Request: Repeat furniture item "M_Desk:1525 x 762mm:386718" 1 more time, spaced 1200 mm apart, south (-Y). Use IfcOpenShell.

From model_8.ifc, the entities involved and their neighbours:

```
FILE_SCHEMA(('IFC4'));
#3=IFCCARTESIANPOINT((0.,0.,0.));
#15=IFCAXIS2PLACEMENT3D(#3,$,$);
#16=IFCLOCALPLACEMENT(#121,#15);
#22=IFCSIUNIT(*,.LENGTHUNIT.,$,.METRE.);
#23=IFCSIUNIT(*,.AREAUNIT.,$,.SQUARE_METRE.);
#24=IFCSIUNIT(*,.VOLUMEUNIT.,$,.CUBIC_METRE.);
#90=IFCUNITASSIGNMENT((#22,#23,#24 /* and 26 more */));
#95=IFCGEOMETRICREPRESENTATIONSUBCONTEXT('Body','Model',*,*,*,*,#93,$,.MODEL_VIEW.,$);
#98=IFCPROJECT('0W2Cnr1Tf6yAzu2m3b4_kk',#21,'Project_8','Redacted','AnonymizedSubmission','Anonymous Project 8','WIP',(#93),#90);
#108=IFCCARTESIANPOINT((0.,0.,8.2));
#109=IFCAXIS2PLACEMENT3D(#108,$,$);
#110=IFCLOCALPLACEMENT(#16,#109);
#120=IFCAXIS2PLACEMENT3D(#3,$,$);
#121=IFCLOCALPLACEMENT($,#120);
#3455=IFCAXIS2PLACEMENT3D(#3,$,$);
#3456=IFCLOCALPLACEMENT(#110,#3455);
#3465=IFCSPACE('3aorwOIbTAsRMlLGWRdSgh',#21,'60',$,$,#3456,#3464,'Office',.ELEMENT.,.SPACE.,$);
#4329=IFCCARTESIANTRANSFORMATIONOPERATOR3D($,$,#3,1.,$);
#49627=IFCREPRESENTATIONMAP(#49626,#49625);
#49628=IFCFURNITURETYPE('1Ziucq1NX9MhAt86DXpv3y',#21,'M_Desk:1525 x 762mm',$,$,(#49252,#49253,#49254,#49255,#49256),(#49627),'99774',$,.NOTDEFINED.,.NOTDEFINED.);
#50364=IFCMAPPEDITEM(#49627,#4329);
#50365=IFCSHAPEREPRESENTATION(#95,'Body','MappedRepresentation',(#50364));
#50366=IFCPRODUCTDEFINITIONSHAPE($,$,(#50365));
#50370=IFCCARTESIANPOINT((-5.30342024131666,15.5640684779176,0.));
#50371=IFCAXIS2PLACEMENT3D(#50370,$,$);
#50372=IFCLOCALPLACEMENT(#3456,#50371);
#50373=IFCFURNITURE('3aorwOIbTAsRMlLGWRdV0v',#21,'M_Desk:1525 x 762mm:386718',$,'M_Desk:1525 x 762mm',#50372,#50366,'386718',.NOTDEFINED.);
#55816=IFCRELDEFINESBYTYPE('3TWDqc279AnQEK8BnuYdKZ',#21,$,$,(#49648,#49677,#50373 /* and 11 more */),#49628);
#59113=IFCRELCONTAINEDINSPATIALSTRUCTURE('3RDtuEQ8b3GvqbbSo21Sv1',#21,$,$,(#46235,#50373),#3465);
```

```python
import numpy as np
import ifcopenshell
import ifcopenshell.api.geometry
import ifcopenshell.api.root
import ifcopenshell.util.element
import ifcopenshell.util.placement
import ifcopenshell.util.unit

model = ifcopenshell.open("model_8.ifc")
unit_scale = ifcopenshell.util.unit.calculate_unit_scale(model)


def reuse_history(source, copy):
    """copy_class also copies each property set's owner history, people and application; keep the originals."""
    for rel in copy.IsDefinedBy:
        if rel.is_a("IfcRelDefinesByProperties") and (history := rel.RelatingPropertyDefinition.OwnerHistory):
            rel.RelatingPropertyDefinition.OwnerHistory = source.OwnerHistory
            ifcopenshell.util.element.remove_deep2(model, history)


source = model.by_id(50373)
base = ifcopenshell.util.placement.get_local_placement(source.ObjectPlacement)
step = np.array([0.0, -1.0, 0.0]) * 1.2 / unit_scale

for i in range(1, 2):
    copy = ifcopenshell.api.root.copy_class(model, product=source)
    copy.Representation = ifcopenshell.util.element.copy_deep(
        model, source.Representation, exclude=["IfcGeometricRepresentationContext", "IfcRepresentationMap"]
    )
    copy.Name = "M_Desk:1525 x 762mm"
    copy.Tag = None
    reuse_history(source, copy)
    matrix = base.copy()
    matrix[:3, 3] += i * step
    print("added at", matrix[:3, 3].round(3) + 0.0)
    ifcopenshell.api.geometry.edit_object_placement(model, product=copy, matrix=matrix, is_si=False)

model.write("model_8_updated.ifc")
```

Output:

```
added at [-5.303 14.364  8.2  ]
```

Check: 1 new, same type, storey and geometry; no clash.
